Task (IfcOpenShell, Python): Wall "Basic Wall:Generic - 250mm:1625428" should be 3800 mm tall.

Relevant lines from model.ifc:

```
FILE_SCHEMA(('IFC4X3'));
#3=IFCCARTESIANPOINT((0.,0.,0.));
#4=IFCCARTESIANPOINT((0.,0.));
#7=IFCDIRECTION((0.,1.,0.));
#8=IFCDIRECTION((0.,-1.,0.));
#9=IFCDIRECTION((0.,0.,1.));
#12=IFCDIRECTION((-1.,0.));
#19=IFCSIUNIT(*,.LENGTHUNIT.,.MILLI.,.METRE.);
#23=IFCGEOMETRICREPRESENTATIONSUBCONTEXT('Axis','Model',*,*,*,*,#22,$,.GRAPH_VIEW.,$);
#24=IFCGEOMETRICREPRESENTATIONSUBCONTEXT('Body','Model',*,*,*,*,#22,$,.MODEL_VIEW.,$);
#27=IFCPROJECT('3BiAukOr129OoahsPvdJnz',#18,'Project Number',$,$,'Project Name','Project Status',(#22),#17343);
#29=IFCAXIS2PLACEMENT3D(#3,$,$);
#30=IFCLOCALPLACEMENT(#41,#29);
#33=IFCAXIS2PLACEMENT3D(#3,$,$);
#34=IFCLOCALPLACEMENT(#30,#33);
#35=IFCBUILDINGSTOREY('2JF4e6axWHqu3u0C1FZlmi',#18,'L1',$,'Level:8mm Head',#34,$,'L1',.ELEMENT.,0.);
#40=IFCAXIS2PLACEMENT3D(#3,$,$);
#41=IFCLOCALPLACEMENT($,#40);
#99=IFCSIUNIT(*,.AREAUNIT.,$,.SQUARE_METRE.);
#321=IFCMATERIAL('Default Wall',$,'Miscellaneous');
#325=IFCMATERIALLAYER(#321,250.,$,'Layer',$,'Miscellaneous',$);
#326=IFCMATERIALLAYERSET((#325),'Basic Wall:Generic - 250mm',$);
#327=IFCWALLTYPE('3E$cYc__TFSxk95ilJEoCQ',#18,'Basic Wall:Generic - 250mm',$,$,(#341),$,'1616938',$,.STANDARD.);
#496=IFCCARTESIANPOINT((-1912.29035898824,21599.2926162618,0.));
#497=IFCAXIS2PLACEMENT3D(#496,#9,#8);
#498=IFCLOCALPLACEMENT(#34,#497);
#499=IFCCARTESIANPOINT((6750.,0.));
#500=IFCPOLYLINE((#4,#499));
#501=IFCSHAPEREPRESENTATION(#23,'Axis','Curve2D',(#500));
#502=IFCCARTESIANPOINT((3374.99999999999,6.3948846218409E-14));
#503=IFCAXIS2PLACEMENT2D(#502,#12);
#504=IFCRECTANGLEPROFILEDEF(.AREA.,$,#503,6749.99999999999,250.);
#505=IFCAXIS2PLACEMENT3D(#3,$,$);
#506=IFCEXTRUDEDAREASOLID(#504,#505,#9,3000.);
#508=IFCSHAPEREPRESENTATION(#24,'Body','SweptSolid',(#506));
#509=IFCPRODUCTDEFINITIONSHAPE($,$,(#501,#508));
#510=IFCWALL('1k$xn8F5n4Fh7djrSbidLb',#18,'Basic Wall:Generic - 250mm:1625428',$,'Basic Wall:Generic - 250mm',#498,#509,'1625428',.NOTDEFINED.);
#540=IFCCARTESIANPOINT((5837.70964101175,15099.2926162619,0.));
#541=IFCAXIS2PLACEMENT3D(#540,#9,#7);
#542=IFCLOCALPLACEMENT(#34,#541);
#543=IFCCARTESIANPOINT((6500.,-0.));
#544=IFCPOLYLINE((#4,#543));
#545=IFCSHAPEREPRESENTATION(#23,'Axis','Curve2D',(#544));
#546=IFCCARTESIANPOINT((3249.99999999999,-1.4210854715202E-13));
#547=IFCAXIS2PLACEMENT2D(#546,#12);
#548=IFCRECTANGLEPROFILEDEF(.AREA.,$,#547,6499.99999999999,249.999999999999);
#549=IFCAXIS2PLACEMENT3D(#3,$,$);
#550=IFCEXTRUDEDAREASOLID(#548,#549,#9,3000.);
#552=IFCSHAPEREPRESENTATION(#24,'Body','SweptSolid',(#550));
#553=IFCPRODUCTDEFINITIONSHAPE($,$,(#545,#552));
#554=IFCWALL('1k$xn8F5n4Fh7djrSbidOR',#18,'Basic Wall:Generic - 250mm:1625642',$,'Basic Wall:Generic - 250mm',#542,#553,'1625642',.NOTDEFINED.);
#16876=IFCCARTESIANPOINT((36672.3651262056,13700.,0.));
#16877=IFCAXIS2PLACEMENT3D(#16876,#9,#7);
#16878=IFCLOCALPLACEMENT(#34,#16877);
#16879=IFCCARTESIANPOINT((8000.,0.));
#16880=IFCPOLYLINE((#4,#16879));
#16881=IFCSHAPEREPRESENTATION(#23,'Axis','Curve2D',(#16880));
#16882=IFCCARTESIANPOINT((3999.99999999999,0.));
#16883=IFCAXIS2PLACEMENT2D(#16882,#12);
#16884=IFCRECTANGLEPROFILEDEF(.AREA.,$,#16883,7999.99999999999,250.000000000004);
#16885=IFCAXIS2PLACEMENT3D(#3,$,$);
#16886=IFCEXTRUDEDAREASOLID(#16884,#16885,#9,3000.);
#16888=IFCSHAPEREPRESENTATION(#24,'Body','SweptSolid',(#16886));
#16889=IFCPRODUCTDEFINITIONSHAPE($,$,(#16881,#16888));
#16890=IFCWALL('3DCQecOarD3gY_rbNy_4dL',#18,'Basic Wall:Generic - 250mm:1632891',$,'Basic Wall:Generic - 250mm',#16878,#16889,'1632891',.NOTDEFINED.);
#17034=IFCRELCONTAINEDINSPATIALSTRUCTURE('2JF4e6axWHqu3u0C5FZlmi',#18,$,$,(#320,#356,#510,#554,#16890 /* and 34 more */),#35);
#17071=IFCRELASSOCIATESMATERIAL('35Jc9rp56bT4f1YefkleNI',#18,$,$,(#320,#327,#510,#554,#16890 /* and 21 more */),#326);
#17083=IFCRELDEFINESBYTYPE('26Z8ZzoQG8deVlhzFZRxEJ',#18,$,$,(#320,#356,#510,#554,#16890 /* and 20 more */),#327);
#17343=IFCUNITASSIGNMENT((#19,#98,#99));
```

```python
import ifcopenshell
import ifcopenshell.geom
import ifcopenshell.util.representation
import ifcopenshell.util.shape
import ifcopenshell.util.unit

model = ifcopenshell.open("model.ifc")
unit_scale = ifcopenshell.util.unit.calculate_unit_scale(model)
settings = ifcopenshell.geom.settings()


def volume(element):
    """Net volume in cubic metres, openings subtracted."""
    shape = ifcopenshell.geom.create_shape(settings, element)
    return ifcopenshell.util.shape.get_volume(shape.geometry)


wall = model.by_guid("1k$xn8F5n4Fh7djrSbidLb")
before = volume(wall)

body = ifcopenshell.util.representation.get_representation(wall, "Model", "Body")
solid = body.Items[0]
old_height = solid.Depth
solid.Depth = 3.8 / unit_scale
after = volume(wall)

print(f"height {old_height:g} -> {solid.Depth:g}, volume {before:.3f} -> {after:.3f} m3")

model.write("model_v2.ifc")
```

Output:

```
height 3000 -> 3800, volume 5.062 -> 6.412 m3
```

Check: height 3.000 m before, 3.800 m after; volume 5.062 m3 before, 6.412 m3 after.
